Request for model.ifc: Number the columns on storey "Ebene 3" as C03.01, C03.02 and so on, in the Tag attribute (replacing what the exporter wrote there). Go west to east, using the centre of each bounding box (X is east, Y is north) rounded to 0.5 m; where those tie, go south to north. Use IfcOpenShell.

First a look at what the model holds.

```python
import ifcopenshell
import ifcopenshell.util.element
import ifcopenshell.util.placement

model = ifcopenshell.open("model.ifc")
print(model.schema)
storey = next(s for s in model.by_type("IfcBuildingStorey") if s.Name == "Ebene 3")
columns = [e for e in ifcopenshell.util.element.get_decomposition(storey) if e.is_a("IfcColumn")]
for e in sorted(columns, key=lambda e: e.id()):
    origin = ifcopenshell.util.placement.get_local_placement(e.ObjectPlacement)[:3, 3]
    print(e.id(), e.Tag, e.Name, origin.round(2) + 0.0, sep=" | ")
```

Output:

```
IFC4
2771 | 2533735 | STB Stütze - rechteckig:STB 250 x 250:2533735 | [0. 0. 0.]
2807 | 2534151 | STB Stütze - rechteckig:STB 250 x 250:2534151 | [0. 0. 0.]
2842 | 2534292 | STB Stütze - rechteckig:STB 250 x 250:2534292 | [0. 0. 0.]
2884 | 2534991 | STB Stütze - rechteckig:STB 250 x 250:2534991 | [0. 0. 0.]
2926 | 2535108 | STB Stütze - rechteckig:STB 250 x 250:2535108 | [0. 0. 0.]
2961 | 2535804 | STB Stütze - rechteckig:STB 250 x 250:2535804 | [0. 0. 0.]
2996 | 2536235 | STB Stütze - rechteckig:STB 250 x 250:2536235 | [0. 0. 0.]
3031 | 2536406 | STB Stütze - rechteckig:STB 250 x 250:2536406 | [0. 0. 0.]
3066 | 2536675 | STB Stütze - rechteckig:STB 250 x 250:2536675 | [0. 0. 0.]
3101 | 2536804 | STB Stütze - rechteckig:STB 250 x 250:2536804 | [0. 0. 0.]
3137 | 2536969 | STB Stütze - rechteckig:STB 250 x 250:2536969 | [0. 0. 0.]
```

```python
import ifcopenshell
import ifcopenshell.geom
import ifcopenshell.util.element
import ifcopenshell.util.shape

model = ifcopenshell.open("model.ifc")
settings = ifcopenshell.geom.settings()
settings.set("use-world-coords", True)


def centre(element):
    shape = ifcopenshell.geom.create_shape(settings, element)
    return ifcopenshell.util.shape.get_bbox_centroid(shape.geometry)


storey = next(s for s in model.by_type("IfcBuildingStorey") if s.Name == "Ebene 3")
columns = [e for e in ifcopenshell.util.element.get_decomposition(storey) if e.is_a("IfcColumn")]

# Insertion points can sit at a corner or the storey origin, so sort by the geometry (in metres).
centres = {e: centre(e) for e in columns}
columns.sort(key=lambda e: (round(centres[e][0] / 0.5), centres[e][1]))

for i, e in enumerate(columns, start=1):
    number = f"C03.{i:02d}"
    e.Tag = number
    print(e.id(), number)

model.write("model_updated.ifc")
```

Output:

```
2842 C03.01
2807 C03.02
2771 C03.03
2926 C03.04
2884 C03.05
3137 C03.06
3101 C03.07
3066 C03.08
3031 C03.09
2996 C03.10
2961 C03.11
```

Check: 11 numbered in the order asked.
